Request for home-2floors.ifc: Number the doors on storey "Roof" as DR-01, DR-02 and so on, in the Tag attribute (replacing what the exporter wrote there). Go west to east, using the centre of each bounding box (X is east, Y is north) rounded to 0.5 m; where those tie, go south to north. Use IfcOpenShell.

First a look at what the model holds.

```python
import ifcopenshell
import ifcopenshell.util.element
import ifcopenshell.util.placement

model = ifcopenshell.open("home-2floors.ifc")
print(model.schema)
storey = next(s for s in model.by_type("IfcBuildingStorey") if s.Name == "Roof")
doors = [e for e in ifcopenshell.util.element.get_decomposition(storey) if e.is_a("IfcDoor")]
for e in sorted(doors, key=lambda e: e.id()):
    origin = ifcopenshell.util.placement.get_local_placement(e.ObjectPlacement)[:3, 3]
    print(e.id(), e.Tag, e.Name, origin.round(2) + 0.0, sep=" | ")
```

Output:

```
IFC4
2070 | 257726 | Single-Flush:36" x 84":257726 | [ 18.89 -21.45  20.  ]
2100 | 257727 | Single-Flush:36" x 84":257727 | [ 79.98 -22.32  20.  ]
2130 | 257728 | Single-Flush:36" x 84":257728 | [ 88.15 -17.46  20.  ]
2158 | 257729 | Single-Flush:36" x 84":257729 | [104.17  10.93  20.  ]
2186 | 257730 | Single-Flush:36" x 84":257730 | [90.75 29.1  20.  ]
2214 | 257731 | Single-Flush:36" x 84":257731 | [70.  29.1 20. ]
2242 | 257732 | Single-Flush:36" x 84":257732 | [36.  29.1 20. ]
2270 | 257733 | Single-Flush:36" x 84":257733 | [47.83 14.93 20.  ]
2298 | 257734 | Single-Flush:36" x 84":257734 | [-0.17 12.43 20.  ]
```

```python
import ifcopenshell
import ifcopenshell.geom
import ifcopenshell.util.element
import ifcopenshell.util.shape

model = ifcopenshell.open("home-2floors.ifc")
settings = ifcopenshell.geom.settings()
settings.set("use-world-coords", True)


def centre(element):
    shape = ifcopenshell.geom.create_shape(settings, element)
    return ifcopenshell.util.shape.get_bbox_centroid(shape.geometry)


storey = next(s for s in model.by_type("IfcBuildingStorey") if s.Name == "Roof")
doors = [e for e in ifcopenshell.util.element.get_decomposition(storey) if e.is_a("IfcDoor")]

# Insertion points can sit at a corner or the storey origin, so sort by the geometry (in metres).
centres = {e: centre(e) for e in doors}
doors.sort(key=lambda e: (round(centres[e][0] / 0.5), centres[e][1]))

for i, e in enumerate(doors, start=1):
    number = f"DR-{i:02d}"
    e.Tag = number
    print(e.id(), number)

model.write("home-2floors-out.ifc")
```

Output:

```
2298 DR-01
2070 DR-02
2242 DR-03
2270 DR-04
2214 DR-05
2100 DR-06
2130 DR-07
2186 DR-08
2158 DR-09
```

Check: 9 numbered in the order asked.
